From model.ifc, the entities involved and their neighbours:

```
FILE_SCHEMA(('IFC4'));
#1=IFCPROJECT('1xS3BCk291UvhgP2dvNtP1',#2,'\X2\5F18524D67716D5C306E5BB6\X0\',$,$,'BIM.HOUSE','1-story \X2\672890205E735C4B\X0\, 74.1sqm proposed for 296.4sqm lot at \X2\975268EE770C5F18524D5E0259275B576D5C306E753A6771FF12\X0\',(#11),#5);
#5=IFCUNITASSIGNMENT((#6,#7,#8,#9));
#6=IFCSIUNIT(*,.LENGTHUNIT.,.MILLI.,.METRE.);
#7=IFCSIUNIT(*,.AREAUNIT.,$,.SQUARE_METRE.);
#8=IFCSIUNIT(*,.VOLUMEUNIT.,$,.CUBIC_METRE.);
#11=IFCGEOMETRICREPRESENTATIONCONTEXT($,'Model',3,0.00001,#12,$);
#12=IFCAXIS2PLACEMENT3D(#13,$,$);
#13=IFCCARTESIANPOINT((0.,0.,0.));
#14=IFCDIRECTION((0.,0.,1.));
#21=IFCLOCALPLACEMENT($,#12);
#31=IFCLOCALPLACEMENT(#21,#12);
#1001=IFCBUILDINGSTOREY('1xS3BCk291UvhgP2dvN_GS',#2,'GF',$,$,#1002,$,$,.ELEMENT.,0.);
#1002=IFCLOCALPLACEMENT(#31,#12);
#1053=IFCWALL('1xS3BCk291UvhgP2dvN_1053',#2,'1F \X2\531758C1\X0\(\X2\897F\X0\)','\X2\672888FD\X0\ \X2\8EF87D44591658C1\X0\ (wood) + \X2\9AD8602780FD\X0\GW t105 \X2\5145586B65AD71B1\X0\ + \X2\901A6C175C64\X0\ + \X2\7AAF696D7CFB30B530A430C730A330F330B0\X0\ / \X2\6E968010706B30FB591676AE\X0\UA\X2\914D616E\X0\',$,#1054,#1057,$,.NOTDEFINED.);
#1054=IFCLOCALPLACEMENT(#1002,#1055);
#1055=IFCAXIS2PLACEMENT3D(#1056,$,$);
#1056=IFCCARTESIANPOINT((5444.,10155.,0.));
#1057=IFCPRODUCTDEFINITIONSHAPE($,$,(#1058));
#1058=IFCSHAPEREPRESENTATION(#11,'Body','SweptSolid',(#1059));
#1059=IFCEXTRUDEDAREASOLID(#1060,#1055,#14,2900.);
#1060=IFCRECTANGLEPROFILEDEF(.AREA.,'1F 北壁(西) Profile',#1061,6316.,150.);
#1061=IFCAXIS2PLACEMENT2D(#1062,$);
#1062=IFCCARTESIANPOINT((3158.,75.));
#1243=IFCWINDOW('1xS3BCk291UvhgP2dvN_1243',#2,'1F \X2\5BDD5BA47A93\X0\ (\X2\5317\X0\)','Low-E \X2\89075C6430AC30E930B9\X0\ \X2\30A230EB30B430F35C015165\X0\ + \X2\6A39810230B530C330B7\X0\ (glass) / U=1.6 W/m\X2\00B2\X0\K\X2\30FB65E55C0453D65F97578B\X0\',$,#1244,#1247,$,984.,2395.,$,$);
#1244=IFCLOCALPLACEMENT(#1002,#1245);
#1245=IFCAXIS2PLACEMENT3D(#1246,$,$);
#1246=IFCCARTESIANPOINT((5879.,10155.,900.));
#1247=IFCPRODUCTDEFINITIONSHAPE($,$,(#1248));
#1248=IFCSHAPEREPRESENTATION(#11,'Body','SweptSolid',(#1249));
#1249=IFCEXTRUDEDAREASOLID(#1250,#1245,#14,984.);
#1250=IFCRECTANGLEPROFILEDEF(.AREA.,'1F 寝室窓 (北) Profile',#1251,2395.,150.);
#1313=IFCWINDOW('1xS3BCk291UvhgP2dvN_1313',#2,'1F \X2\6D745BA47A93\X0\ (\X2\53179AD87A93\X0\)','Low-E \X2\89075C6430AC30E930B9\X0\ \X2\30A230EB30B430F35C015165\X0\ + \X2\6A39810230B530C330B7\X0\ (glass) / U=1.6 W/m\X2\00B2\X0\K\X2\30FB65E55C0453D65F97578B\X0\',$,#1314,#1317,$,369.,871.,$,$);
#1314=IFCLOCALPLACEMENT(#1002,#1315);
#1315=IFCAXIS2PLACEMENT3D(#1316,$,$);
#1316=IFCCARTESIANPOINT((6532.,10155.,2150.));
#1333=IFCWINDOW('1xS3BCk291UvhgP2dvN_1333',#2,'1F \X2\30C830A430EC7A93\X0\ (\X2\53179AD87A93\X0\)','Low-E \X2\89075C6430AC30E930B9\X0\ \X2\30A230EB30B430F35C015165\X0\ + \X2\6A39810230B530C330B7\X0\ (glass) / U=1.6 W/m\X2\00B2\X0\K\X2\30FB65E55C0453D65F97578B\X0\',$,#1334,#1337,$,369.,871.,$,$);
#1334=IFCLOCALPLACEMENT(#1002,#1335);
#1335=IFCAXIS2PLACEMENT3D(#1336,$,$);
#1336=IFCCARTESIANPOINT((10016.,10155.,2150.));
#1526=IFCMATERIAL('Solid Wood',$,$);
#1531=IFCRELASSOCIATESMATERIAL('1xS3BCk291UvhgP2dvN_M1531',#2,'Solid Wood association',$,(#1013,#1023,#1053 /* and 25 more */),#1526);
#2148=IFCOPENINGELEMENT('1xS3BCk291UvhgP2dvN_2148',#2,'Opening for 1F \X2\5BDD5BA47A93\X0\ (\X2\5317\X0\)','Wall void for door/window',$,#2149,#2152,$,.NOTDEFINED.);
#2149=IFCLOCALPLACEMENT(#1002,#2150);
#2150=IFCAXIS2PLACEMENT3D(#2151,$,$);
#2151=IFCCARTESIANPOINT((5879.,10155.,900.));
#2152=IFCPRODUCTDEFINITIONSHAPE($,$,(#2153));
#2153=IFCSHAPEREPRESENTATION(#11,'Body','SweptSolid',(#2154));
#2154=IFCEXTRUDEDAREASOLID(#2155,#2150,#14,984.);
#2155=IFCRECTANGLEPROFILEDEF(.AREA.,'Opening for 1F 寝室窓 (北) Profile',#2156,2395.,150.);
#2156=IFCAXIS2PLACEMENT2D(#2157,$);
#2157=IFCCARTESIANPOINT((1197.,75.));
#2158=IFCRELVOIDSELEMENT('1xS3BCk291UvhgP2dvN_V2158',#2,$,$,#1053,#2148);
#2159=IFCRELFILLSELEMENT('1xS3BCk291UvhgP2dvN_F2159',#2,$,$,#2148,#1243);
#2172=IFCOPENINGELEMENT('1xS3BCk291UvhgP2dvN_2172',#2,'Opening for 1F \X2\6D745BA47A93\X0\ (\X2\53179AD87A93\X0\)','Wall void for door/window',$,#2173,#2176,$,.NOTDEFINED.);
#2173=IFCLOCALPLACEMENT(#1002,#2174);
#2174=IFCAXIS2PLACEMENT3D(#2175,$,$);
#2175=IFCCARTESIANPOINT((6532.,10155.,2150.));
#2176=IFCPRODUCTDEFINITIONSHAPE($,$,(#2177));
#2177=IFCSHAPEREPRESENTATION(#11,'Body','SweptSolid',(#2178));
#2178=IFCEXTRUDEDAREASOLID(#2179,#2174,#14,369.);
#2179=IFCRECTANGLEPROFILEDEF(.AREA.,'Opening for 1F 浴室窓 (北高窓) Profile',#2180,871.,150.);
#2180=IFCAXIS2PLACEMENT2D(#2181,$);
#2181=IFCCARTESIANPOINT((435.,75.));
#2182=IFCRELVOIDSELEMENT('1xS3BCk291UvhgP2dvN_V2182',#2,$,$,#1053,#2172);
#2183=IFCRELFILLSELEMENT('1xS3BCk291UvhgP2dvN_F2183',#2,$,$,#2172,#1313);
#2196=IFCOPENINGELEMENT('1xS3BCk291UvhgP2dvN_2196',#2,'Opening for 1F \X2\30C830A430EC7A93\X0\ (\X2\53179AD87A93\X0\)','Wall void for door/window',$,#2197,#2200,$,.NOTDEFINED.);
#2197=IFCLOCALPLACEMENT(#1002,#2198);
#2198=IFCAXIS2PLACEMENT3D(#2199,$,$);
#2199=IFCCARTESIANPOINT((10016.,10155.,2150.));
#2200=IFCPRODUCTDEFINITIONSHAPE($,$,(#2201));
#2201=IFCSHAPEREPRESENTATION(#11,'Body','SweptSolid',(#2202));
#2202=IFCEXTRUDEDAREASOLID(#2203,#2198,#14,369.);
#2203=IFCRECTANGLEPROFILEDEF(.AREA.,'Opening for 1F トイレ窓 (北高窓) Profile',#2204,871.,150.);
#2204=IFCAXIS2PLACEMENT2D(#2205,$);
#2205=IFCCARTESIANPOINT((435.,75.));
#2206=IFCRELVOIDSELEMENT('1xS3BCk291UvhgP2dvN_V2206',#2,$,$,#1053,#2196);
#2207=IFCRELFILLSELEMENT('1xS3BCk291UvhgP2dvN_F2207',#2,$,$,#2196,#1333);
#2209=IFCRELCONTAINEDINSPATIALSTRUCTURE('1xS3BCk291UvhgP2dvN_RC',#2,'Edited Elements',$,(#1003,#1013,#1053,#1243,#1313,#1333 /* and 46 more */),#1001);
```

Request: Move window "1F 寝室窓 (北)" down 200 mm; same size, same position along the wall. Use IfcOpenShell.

```python
import numpy as np
import ifcopenshell
import ifcopenshell.api.geometry
import ifcopenshell.util.placement
import ifcopenshell.util.unit

model = ifcopenshell.open("model.ifc")
unit_scale = ifcopenshell.util.unit.calculate_unit_scale(model)

window = model.by_guid("1xS3BCk291UvhgP2dvN_1243")
opening = window.FillsVoids[0].RelatingOpeningElement
dz = -0.2 / unit_scale

shift = np.array([0.0, 0.0, dz])
# The window is not placed relative to its opening, so move both.
for product in (opening, window):
    matrix = ifcopenshell.util.placement.get_local_placement(product.ObjectPlacement)
    matrix[:3, 3] += shift
    ifcopenshell.api.geometry.edit_object_placement(model, product=product, matrix=matrix, is_si=False)

print(f"moved by {dz * unit_scale:+.3f} m")

model.write("model_v2.ifc")
```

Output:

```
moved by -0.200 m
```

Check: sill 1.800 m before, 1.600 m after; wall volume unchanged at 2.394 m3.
